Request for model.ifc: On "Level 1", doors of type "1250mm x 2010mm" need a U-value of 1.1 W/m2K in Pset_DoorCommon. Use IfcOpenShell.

First a look at what the model holds.

```python
import ifcopenshell
import ifcopenshell.util.element

model = ifcopenshell.open("model.ifc")
print(model.schema)
storey = next(s for s in model.by_type("IfcBuildingStorey") if s.Name == "Level 1")
doors = [e for e in ifcopenshell.util.element.get_decomposition(storey) if e.is_a("IfcDoor")]
seen = {}
for e in doors:
    element_type = ifcopenshell.util.element.get_type(e)
    key = (element_type.Name if element_type != e and element_type else None, ifcopenshell.util.element.get_pset(e, "Pset_DoorCommon", "ThermalTransmittance"))
    seen[key] = seen.get(key, 0) + 1
for (name, value), count in sorted(seen.items(), key=str):
    print(count, "x", name, "|", value)
```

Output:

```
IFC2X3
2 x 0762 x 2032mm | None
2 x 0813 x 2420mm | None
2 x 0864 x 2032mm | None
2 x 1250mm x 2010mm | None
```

```python
import ifcopenshell
import ifcopenshell.api.pset
import ifcopenshell.util.element

model = ifcopenshell.open("model.ifc")

storey = next(s for s in model.by_type("IfcBuildingStorey") if s.Name == "Level 1")
doors = [e for e in ifcopenshell.util.element.get_decomposition(storey) if e.is_a("IfcDoor")]

count = 0
for e in doors:
    element_type = ifcopenshell.util.element.get_type(e)
    if element_type in (None, e) or element_type.Name != "1250mm x 2010mm":
        continue
    # add_pset returns the element's existing set when there is one.
    pset = ifcopenshell.api.pset.add_pset(model, product=e, name="Pset_DoorCommon")
    ifcopenshell.api.pset.edit_pset(model, pset=pset, properties={"ThermalTransmittance": 1.1})
    count += 1

print(count, "doors updated")

model.write("model_updated.ifc")
```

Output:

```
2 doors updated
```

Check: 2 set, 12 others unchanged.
